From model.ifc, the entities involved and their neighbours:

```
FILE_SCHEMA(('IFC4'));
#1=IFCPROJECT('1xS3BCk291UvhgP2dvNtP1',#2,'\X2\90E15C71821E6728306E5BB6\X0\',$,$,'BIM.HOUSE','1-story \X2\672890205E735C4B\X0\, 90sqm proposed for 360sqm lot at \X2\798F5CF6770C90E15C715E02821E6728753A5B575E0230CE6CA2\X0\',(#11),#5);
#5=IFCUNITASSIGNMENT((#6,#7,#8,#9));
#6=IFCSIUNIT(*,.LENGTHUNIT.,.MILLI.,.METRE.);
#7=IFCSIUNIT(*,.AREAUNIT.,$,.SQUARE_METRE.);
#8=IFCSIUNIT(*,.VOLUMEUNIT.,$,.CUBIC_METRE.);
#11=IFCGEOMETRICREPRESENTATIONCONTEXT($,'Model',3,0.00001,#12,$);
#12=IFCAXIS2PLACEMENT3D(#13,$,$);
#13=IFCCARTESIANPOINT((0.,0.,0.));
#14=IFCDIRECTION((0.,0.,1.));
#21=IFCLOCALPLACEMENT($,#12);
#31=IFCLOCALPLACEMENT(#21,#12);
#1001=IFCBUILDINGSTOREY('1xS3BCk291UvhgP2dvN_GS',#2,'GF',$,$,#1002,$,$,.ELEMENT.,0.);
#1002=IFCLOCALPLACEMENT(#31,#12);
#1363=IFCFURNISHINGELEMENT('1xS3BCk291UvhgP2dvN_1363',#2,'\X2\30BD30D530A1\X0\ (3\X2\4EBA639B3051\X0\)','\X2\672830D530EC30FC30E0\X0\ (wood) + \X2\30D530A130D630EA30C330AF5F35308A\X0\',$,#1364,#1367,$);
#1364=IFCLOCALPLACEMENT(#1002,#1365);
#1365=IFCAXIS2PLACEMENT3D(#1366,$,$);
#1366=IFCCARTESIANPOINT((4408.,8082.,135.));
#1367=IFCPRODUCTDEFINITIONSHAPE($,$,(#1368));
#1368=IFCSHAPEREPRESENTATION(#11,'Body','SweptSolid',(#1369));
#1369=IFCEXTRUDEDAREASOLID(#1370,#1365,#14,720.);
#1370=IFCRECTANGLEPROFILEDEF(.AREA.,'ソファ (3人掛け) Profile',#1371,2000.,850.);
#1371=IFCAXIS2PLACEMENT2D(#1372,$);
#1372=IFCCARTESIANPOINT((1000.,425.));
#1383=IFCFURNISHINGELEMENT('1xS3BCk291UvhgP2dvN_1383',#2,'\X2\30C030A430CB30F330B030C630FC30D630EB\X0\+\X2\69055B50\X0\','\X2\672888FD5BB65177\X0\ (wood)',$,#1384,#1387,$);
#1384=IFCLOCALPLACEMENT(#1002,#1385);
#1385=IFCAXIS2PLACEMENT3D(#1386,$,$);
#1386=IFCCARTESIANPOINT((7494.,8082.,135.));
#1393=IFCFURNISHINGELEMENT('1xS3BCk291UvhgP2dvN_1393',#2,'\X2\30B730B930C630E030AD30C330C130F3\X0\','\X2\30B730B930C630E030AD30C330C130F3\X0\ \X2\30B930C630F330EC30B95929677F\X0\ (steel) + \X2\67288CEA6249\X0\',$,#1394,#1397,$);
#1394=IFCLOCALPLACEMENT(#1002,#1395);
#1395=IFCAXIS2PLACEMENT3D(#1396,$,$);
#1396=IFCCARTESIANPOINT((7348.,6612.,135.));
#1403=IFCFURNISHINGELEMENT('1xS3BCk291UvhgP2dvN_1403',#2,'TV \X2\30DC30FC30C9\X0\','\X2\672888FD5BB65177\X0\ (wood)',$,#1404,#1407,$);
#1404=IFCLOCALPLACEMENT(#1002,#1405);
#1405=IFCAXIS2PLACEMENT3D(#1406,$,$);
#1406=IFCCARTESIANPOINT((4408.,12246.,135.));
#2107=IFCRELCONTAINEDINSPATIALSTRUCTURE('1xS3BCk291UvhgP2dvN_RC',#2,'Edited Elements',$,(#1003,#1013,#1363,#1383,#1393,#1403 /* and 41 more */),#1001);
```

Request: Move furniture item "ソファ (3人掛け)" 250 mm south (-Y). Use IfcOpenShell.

```python
import ifcopenshell
import ifcopenshell.api.geometry
import ifcopenshell.util.placement

model = ifcopenshell.open("model.ifc")

item = model.by_guid("1xS3BCk291UvhgP2dvN_1363")
matrix = ifcopenshell.util.placement.get_local_placement(item.ObjectPlacement)
matrix[1, 3] -= 250.0
ifcopenshell.api.geometry.edit_object_placement(model, product=item, matrix=matrix, is_si=False)

print(ifcopenshell.util.placement.get_local_placement(item.ObjectPlacement).round(3) + 0.0)

model.write("model-out.ifc")
```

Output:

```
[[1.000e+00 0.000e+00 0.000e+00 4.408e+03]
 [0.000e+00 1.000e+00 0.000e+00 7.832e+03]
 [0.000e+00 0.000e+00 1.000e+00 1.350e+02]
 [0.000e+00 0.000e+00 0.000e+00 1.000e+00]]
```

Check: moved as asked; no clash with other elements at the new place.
